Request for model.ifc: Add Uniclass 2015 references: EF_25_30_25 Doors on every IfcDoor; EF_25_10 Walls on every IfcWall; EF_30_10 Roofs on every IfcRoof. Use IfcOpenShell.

First a look at what the model holds.

```python
import ifcopenshell

model = ifcopenshell.open("model.ifc")
print(model.schema)
print("classifications:", [c.Name for c in model.by_type("IfcClassification")])
for ifc_class in ("IfcDoor", "IfcRoof", "IfcStair", "IfcWall", "IfcWindow"):
    print(ifc_class, len(model.by_type(ifc_class)))
```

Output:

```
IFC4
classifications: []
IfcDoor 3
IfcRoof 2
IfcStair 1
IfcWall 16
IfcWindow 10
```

```python
import ifcopenshell
import ifcopenshell.api.classification

model = ifcopenshell.open("model.ifc")

system = ifcopenshell.api.classification.add_classification(model, classification="Uniclass 2015")

codes = {
    "IfcDoor": ("EF_25_30_25", "Doors"),
    "IfcWall": ("EF_25_10", "Walls"),
    "IfcRoof": ("EF_30_10", "Roofs"),
}
for ifc_class, (code, name) in codes.items():
    products = model.by_type(ifc_class)
    ifcopenshell.api.classification.add_reference(
        model, products=products, classification=system, identification=code, name=name
    )
    print(code, len(products))

model.write("model_edited.ifc")
```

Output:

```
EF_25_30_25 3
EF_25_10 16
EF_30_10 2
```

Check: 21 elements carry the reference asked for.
